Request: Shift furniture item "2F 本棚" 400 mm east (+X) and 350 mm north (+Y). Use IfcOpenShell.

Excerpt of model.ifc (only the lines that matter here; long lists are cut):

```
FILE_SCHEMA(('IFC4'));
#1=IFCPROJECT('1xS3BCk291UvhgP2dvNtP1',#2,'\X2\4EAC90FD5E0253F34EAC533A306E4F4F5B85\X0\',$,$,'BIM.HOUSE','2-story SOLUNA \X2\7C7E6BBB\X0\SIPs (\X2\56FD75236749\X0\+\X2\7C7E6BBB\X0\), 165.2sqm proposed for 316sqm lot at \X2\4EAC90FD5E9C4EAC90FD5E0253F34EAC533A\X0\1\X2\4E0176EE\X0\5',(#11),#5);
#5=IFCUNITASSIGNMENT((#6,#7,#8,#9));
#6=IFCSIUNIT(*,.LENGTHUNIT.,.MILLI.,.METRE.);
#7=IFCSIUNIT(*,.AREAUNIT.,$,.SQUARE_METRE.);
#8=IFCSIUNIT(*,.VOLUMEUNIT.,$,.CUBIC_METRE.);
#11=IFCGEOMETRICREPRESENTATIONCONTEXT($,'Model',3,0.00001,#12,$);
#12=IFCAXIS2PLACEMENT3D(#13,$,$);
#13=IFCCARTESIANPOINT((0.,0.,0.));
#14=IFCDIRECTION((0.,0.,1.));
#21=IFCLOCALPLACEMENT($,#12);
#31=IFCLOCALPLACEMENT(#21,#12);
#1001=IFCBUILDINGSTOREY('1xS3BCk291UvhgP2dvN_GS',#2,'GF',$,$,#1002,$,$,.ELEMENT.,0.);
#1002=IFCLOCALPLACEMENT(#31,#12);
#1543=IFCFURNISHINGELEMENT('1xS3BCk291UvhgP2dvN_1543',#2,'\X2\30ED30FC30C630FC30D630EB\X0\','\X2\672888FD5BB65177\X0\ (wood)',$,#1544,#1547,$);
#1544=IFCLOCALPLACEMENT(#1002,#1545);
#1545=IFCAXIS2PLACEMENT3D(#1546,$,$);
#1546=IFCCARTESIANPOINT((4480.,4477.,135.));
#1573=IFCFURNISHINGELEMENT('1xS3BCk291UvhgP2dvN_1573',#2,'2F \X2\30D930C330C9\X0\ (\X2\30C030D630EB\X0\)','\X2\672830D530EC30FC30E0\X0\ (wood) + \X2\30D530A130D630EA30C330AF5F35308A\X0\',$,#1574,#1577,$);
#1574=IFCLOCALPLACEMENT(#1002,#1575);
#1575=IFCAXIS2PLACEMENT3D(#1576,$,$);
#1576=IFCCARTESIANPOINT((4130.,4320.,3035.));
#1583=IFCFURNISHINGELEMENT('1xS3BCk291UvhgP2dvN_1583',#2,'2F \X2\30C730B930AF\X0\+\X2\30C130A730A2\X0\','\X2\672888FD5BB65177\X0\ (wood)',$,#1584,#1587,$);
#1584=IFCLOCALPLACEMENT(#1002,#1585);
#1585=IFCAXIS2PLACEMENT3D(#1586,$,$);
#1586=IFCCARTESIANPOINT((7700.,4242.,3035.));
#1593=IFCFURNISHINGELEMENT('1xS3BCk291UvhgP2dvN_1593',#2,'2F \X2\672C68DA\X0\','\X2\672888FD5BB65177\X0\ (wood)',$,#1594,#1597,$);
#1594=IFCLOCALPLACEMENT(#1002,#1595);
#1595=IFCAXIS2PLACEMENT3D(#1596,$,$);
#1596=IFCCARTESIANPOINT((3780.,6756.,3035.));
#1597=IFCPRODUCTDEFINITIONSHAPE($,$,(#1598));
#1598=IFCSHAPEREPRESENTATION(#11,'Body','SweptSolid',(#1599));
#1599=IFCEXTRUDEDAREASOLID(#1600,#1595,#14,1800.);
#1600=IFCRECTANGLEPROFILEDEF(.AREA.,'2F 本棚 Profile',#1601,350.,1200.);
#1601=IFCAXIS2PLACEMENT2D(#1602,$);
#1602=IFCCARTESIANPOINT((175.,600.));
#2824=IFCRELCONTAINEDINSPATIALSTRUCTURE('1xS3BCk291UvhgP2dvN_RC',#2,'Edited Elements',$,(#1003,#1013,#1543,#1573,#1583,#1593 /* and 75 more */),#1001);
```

```python
import ifcopenshell
import ifcopenshell.api.geometry
import ifcopenshell.util.placement

model = ifcopenshell.open("model.ifc")

item = model.by_id(1593)
matrix = ifcopenshell.util.placement.get_local_placement(item.ObjectPlacement)
matrix[0, 3] += 400.0
matrix[1, 3] += 350.0
ifcopenshell.api.geometry.edit_object_placement(model, product=item, matrix=matrix, is_si=False)

print(ifcopenshell.util.placement.get_local_placement(item.ObjectPlacement).round(3) + 0.0)

model.write("model_updated.ifc")
```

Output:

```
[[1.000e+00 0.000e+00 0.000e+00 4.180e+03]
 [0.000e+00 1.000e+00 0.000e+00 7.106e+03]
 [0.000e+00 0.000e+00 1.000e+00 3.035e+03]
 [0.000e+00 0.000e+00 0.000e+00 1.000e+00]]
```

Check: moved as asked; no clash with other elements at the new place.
